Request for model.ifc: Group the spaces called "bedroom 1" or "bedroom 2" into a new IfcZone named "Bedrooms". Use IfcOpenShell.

First a look at what the model holds.

```python
import ifcopenshell

model = ifcopenshell.open("model.ifc")
print(model.schema)
seen = {}
for space in model.by_type("IfcSpace"):
    seen[space.LongName] = seen.get(space.LongName, 0) + 1
for name, count in sorted(seen.items(), key=str):
    print(count, "x", name)
print("zones:", [z.Name for z in model.by_type("IfcZone")][:20])
```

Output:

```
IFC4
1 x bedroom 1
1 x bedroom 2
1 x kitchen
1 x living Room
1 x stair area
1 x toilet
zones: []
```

```python
import ifcopenshell
import ifcopenshell.api.group
import ifcopenshell.api.root

model = ifcopenshell.open("model.ifc")

names = {"bedroom 1", "bedroom 2"}
spaces = [s for s in model.by_type("IfcSpace") if s.LongName in names]

zone = ifcopenshell.api.root.create_entity(model, ifc_class="IfcZone", name="Bedrooms")
ifcopenshell.api.group.assign_group(model, products=spaces, group=zone)
print(len(spaces), "spaces in", zone.Name)

model.write("model_rev.ifc")
```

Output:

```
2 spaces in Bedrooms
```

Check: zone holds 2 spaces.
